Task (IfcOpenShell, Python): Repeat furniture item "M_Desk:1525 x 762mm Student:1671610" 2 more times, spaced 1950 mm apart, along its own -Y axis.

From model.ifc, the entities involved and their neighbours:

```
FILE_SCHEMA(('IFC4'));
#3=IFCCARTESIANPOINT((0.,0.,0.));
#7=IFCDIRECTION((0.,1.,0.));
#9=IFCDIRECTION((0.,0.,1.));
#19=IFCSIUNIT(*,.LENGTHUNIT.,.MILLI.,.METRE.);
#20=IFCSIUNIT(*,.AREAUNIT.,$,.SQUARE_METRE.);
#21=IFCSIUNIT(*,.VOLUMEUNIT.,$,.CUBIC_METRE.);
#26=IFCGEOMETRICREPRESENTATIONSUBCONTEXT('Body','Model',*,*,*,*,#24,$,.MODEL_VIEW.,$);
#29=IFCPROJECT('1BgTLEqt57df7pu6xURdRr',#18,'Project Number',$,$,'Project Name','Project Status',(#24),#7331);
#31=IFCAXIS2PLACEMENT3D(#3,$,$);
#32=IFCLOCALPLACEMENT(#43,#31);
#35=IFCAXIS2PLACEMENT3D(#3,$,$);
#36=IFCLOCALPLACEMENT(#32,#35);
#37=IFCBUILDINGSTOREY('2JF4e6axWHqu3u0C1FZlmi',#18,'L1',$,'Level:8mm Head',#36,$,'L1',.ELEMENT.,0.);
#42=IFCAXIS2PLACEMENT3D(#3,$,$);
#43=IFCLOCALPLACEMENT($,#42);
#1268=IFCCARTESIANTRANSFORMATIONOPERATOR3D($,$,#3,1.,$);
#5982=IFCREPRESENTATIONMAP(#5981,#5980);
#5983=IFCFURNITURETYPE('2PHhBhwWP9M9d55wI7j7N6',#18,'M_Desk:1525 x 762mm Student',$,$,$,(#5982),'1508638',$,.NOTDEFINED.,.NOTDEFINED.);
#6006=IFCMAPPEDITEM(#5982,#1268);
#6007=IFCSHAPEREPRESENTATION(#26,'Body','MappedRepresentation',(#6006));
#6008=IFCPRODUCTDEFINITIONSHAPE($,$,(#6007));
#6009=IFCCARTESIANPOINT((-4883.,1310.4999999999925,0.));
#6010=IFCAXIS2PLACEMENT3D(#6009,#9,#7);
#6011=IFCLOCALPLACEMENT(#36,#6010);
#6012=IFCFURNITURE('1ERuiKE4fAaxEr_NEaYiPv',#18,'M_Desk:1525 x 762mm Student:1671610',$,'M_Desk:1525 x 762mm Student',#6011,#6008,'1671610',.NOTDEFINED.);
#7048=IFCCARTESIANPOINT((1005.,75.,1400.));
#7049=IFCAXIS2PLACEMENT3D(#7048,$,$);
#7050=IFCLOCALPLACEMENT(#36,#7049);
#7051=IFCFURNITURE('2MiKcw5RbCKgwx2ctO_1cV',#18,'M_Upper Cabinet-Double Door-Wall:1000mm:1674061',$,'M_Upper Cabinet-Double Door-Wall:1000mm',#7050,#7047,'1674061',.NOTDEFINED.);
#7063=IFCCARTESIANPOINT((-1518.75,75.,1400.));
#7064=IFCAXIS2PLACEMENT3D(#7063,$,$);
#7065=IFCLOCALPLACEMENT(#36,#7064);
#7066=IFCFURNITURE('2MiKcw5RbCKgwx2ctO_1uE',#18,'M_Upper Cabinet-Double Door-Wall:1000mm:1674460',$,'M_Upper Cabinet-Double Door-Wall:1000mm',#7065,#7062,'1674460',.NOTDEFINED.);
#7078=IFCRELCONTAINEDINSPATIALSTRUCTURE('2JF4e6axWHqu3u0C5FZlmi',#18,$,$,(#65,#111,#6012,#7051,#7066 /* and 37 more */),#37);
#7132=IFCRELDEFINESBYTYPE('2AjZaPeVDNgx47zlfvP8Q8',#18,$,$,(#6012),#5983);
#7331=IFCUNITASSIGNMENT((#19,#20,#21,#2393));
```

```python
import ifcopenshell
import ifcopenshell.api.geometry
import ifcopenshell.api.root
import ifcopenshell.util.element
import ifcopenshell.util.placement
import ifcopenshell.util.unit

model = ifcopenshell.open("model.ifc")
unit_scale = ifcopenshell.util.unit.calculate_unit_scale(model)


def reuse_history(source, copy):
    """copy_class also copies each property set's owner history, people and application; keep the originals."""
    for rel in copy.IsDefinedBy:
        if rel.is_a("IfcRelDefinesByProperties") and (history := rel.RelatingPropertyDefinition.OwnerHistory):
            rel.RelatingPropertyDefinition.OwnerHistory = source.OwnerHistory
            ifcopenshell.util.element.remove_deep2(model, history)


source = model.by_id(6012)
base = ifcopenshell.util.placement.get_local_placement(source.ObjectPlacement)
step = -base[:3, 1] * 1.95 / unit_scale

for i in range(1, 3):
    copy = ifcopenshell.api.root.copy_class(model, product=source)
    copy.Representation = ifcopenshell.util.element.copy_deep(
        model, source.Representation, exclude=["IfcGeometricRepresentationContext", "IfcRepresentationMap"]
    )
    copy.Name = "M_Desk:1525 x 762mm Student"
    copy.Tag = None
    reuse_history(source, copy)
    matrix = base.copy()
    matrix[:3, 3] += i * step
    print("added at", matrix[:3, 3].round(3) + 0.0)
    ifcopenshell.api.geometry.edit_object_placement(model, product=copy, matrix=matrix, is_si=False)

model.write("model_v2.ifc")
```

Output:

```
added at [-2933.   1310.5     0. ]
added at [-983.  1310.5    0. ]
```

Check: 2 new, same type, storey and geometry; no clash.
